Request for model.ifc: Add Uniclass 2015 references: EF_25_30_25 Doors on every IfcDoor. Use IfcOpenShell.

First a look at what the model holds.

```python
import ifcopenshell

model = ifcopenshell.open("model.ifc")
print(model.schema)
print("classifications:", [c.Name for c in model.by_type("IfcClassification")])
for ifc_class in ("IfcDoor", "IfcRoof", "IfcStair", "IfcWall", "IfcWindow"):
    print(ifc_class, len(model.by_type(ifc_class)))
```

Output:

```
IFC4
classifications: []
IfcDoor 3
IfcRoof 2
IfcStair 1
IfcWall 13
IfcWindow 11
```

```python
import ifcopenshell
import ifcopenshell.api.classification

model = ifcopenshell.open("model.ifc")

system = ifcopenshell.api.classification.add_classification(model, classification="Uniclass 2015")

codes = {
    "IfcDoor": ("EF_25_30_25", "Doors"),
}
for ifc_class, (code, name) in codes.items():
    products = model.by_type(ifc_class)
    ifcopenshell.api.classification.add_reference(
        model, products=products, classification=system, identification=code, name=name
    )
    print(code, len(products))

model.write("model_v2.ifc")
```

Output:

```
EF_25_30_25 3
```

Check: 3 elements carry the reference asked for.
